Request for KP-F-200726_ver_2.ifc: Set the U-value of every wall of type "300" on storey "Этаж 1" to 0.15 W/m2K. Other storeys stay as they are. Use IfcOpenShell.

First a look at what the model holds.

```python
import ifcopenshell
import ifcopenshell.util.element

model = ifcopenshell.open("KP-F-200726_ver_2.ifc")
print(model.schema)
storey = next(s for s in model.by_type("IfcBuildingStorey") if s.Name == "Этаж 1")
walls = [e for e in ifcopenshell.util.element.get_decomposition(storey) if e.is_a("IfcWall")]
seen = {}
for e in walls:
    element_type = ifcopenshell.util.element.get_type(e)
    key = (element_type.Name if element_type != e and element_type else None, ifcopenshell.util.element.get_pset(e, "Pset_WallCommon", "ThermalTransmittance"))
    seen[key] = seen.get(key, 0) + 1
for (name, value), count in sorted(seen.items(), key=str):
    print(count, "x", name, "|", value)
```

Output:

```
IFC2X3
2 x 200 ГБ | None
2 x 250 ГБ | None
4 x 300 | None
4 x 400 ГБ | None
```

```python
import ifcopenshell
import ifcopenshell.api.pset
import ifcopenshell.util.element

model = ifcopenshell.open("KP-F-200726_ver_2.ifc")

storey = next(s for s in model.by_type("IfcBuildingStorey") if s.Name == "Этаж 1")
walls = [e for e in ifcopenshell.util.element.get_decomposition(storey) if e.is_a("IfcWall")]

count = 0
for e in walls:
    element_type = ifcopenshell.util.element.get_type(e)
    if element_type in (None, e) or element_type.Name != "300":
        continue
    # add_pset returns the element's existing set when there is one.
    pset = ifcopenshell.api.pset.add_pset(model, product=e, name="Pset_WallCommon")
    ifcopenshell.api.pset.edit_pset(model, pset=pset, properties={"ThermalTransmittance": 0.15})
    count += 1

print(count, "walls updated")

model.write("KP-F-200726_ver_2_rev.ifc")
```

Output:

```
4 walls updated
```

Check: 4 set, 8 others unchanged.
